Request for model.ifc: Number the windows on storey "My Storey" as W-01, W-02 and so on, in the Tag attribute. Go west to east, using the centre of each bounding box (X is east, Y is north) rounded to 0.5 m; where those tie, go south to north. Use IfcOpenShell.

First a look at what the model holds.

```python
import ifcopenshell
import ifcopenshell.util.element
import ifcopenshell.util.placement

model = ifcopenshell.open("model.ifc")
print(model.schema)
storey = next(s for s in model.by_type("IfcBuildingStorey") if s.Name == "My Storey")
windows = [e for e in ifcopenshell.util.element.get_decomposition(storey) if e.is_a("IfcWindow")]
for e in sorted(windows, key=lambda e: e.id()):
    origin = ifcopenshell.util.placement.get_local_placement(e.ObjectPlacement)[:3, 3]
    print(e.id(), e.Tag, e.Name, origin.round(2) + 0.0, sep=" | ")
```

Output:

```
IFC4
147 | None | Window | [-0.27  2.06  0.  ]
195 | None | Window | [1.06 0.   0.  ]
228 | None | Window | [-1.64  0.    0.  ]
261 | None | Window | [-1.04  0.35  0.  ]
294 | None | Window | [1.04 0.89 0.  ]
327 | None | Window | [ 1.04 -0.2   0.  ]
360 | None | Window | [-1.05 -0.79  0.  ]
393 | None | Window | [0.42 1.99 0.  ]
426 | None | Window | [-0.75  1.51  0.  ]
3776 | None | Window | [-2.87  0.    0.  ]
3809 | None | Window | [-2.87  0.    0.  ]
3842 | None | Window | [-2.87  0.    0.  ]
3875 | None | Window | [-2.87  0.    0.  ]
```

```python
import ifcopenshell
import ifcopenshell.geom
import ifcopenshell.util.element
import ifcopenshell.util.shape

model = ifcopenshell.open("model.ifc")
settings = ifcopenshell.geom.settings()
settings.set("use-world-coords", True)


def centre(element):
    shape = ifcopenshell.geom.create_shape(settings, element)
    return ifcopenshell.util.shape.get_bbox_centroid(shape.geometry)


storey = next(s for s in model.by_type("IfcBuildingStorey") if s.Name == "My Storey")
windows = [e for e in ifcopenshell.util.element.get_decomposition(storey) if e.is_a("IfcWindow")]

# Insertion points can sit at a corner or the storey origin, so sort by the geometry (in metres).
centres = {e: centre(e) for e in windows}
windows.sort(key=lambda e: (round(centres[e][0] / 0.5), centres[e][1]))

for i, e in enumerate(windows, start=1):
    number = f"W-{i:02d}"
    e.Tag = number
    print(e.id(), number)

model.write("model_v2.ifc")
```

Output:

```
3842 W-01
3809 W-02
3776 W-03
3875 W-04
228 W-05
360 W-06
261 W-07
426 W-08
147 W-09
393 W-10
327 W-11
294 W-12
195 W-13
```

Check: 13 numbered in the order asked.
